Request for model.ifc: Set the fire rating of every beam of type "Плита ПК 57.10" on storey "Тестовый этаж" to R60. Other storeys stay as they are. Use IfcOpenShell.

First a look at what the model holds.

```python
import ifcopenshell
import ifcopenshell.util.element

model = ifcopenshell.open("model.ifc")
print(model.schema)
storey = next(s for s in model.by_type("IfcBuildingStorey") if s.Name == "Тестовый этаж")
beams = [e for e in ifcopenshell.util.element.get_decomposition(storey) if e.is_a("IfcBeam")]
seen = {}
for e in beams:
    element_type = ifcopenshell.util.element.get_type(e)
    key = (element_type.Name if element_type != e and element_type else None, ifcopenshell.util.element.get_pset(e, "Pset_BeamCommon", "FireRating"))
    seen[key] = seen.get(key, 0) + 1
for (name, value), count in sorted(seen.items(), key=str):
    print(count, "x", name, "|", value)
```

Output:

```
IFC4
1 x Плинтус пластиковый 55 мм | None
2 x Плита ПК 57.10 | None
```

```python
import ifcopenshell
import ifcopenshell.api.pset
import ifcopenshell.util.element

model = ifcopenshell.open("model.ifc")

storey = next(s for s in model.by_type("IfcBuildingStorey") if s.Name == "Тестовый этаж")
beams = [e for e in ifcopenshell.util.element.get_decomposition(storey) if e.is_a("IfcBeam")]

count = 0
for e in beams:
    element_type = ifcopenshell.util.element.get_type(e)
    if element_type in (None, e) or element_type.Name != "Плита ПК 57.10":
        continue
    # add_pset returns the element's existing set when there is one.
    pset = ifcopenshell.api.pset.add_pset(model, product=e, name="Pset_BeamCommon")
    ifcopenshell.api.pset.edit_pset(model, pset=pset, properties={"FireRating": "R60"})
    count += 1

print(count, "beams updated")

model.write("model_edited.ifc")
```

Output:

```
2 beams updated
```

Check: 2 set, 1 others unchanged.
